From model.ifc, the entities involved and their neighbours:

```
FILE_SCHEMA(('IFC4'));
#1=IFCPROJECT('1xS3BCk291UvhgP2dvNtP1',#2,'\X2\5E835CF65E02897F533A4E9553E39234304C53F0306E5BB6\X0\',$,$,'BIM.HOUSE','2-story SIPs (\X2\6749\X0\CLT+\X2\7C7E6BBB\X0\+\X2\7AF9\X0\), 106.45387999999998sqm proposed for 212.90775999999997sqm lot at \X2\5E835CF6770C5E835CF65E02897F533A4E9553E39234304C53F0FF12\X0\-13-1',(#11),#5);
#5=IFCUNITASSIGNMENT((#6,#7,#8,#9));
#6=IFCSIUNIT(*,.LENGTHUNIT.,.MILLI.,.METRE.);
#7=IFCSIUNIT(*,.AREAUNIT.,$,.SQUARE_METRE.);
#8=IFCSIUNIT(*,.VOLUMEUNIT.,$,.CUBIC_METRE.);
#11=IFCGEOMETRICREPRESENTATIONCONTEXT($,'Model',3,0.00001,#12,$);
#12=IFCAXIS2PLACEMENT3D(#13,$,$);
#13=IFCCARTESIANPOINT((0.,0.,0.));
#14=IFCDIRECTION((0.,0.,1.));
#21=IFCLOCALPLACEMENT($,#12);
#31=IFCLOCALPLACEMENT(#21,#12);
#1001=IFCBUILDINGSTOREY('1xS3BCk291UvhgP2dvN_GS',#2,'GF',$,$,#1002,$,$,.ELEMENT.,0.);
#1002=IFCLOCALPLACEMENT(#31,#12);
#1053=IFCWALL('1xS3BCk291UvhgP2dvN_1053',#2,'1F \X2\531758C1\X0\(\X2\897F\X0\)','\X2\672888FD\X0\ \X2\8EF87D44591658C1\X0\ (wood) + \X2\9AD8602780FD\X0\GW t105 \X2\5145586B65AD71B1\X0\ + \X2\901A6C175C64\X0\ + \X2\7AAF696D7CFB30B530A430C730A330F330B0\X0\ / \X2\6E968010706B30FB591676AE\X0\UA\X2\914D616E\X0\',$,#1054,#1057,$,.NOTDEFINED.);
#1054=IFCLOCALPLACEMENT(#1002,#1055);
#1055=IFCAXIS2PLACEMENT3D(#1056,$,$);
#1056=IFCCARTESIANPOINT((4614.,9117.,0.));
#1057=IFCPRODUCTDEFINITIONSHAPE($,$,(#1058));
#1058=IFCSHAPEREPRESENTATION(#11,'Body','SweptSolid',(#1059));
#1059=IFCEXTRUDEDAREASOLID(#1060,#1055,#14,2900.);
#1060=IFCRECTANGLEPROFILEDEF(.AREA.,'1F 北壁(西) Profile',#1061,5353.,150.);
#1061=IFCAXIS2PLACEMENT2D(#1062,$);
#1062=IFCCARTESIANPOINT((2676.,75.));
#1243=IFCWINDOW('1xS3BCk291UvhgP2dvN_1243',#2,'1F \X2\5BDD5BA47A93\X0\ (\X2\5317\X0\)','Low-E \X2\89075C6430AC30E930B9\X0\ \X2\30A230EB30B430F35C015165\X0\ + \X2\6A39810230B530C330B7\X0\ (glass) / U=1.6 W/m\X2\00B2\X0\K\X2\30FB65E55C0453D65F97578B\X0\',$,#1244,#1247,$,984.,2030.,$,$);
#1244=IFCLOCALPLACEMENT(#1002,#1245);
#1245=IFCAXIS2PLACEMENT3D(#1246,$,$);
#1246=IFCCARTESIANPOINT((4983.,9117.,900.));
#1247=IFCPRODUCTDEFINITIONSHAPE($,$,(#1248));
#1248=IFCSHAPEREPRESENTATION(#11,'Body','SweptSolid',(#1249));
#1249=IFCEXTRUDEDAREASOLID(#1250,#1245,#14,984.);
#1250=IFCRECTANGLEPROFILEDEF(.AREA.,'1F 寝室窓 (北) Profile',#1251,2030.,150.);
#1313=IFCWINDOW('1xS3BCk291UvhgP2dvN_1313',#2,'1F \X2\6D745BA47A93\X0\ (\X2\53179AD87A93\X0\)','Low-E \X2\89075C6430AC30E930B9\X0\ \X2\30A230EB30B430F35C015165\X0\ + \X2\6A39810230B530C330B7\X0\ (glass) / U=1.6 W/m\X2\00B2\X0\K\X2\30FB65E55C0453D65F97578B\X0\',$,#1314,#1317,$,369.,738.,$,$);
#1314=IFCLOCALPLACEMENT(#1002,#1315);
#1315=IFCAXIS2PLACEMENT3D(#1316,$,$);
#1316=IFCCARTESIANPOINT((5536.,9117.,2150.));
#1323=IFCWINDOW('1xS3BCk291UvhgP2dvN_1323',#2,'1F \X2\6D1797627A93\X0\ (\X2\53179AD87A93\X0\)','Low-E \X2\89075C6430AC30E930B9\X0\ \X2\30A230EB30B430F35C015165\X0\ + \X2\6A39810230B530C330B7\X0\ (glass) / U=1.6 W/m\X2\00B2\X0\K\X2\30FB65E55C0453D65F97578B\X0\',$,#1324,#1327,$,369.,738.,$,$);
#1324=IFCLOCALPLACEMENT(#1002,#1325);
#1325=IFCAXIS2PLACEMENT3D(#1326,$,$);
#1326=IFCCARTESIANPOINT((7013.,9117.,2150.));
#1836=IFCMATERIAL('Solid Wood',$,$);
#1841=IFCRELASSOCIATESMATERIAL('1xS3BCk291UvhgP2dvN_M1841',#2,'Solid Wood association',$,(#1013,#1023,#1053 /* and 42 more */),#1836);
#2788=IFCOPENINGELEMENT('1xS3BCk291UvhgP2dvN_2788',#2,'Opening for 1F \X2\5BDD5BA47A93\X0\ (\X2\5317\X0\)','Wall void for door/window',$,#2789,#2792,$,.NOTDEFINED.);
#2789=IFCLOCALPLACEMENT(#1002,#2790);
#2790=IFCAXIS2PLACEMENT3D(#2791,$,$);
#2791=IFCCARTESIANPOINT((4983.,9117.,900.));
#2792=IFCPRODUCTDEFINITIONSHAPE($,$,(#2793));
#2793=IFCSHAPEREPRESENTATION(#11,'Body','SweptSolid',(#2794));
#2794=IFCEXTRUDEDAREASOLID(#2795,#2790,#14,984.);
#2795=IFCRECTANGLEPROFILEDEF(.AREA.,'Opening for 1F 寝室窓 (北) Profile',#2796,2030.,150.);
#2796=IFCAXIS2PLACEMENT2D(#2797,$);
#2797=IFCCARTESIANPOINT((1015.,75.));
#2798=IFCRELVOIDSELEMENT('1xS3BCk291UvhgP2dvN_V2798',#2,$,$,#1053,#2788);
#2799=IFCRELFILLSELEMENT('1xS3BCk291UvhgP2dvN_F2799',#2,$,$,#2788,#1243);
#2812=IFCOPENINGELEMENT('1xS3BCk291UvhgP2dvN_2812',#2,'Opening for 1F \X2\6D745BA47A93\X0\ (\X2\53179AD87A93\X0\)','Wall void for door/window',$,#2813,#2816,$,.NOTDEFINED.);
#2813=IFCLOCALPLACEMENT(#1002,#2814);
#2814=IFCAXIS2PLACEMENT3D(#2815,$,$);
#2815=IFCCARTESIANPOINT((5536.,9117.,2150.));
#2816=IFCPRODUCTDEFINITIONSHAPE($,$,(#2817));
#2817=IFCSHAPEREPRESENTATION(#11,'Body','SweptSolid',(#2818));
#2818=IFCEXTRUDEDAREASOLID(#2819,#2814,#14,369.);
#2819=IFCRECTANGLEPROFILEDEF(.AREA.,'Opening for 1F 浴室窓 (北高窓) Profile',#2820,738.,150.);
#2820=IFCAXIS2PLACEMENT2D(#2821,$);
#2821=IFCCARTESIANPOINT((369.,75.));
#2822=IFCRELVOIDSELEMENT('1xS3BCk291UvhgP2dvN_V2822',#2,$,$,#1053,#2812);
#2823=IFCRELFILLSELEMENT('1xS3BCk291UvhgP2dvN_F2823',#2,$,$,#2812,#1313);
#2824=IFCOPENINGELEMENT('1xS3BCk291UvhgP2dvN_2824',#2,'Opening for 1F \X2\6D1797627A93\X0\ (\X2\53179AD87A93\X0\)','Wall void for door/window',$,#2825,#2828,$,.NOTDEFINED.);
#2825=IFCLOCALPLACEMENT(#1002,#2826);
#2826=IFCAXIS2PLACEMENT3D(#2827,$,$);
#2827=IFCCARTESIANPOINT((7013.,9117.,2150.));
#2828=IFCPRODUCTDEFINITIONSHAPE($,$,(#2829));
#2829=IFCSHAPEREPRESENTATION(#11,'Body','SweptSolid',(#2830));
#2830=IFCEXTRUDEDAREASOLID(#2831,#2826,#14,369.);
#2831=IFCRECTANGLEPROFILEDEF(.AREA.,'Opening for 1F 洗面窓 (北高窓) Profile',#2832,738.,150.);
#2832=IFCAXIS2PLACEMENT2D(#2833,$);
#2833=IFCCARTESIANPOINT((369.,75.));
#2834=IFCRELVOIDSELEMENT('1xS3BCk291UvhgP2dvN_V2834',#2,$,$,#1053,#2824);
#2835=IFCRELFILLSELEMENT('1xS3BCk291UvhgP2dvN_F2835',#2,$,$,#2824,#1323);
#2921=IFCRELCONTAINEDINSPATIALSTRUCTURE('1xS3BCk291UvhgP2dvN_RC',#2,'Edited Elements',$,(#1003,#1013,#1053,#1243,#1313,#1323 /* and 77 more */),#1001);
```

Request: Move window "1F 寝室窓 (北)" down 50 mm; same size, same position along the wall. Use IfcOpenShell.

```python
import numpy as np
import ifcopenshell
import ifcopenshell.api.geometry
import ifcopenshell.util.placement
import ifcopenshell.util.unit

model = ifcopenshell.open("model.ifc")
unit_scale = ifcopenshell.util.unit.calculate_unit_scale(model)

window = model.by_id(1243)
opening = window.FillsVoids[0].RelatingOpeningElement
dz = -0.05 / unit_scale

shift = np.array([0.0, 0.0, dz])
# The window is not placed relative to its opening, so move both.
for product in (opening, window):
    matrix = ifcopenshell.util.placement.get_local_placement(product.ObjectPlacement)
    matrix[:3, 3] += shift
    ifcopenshell.api.geometry.edit_object_placement(model, product=product, matrix=matrix, is_si=False)

print(f"moved by {dz * unit_scale:+.3f} m")

model.write("model_rev.ifc")
```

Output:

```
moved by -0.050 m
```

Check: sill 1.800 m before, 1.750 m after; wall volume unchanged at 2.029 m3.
